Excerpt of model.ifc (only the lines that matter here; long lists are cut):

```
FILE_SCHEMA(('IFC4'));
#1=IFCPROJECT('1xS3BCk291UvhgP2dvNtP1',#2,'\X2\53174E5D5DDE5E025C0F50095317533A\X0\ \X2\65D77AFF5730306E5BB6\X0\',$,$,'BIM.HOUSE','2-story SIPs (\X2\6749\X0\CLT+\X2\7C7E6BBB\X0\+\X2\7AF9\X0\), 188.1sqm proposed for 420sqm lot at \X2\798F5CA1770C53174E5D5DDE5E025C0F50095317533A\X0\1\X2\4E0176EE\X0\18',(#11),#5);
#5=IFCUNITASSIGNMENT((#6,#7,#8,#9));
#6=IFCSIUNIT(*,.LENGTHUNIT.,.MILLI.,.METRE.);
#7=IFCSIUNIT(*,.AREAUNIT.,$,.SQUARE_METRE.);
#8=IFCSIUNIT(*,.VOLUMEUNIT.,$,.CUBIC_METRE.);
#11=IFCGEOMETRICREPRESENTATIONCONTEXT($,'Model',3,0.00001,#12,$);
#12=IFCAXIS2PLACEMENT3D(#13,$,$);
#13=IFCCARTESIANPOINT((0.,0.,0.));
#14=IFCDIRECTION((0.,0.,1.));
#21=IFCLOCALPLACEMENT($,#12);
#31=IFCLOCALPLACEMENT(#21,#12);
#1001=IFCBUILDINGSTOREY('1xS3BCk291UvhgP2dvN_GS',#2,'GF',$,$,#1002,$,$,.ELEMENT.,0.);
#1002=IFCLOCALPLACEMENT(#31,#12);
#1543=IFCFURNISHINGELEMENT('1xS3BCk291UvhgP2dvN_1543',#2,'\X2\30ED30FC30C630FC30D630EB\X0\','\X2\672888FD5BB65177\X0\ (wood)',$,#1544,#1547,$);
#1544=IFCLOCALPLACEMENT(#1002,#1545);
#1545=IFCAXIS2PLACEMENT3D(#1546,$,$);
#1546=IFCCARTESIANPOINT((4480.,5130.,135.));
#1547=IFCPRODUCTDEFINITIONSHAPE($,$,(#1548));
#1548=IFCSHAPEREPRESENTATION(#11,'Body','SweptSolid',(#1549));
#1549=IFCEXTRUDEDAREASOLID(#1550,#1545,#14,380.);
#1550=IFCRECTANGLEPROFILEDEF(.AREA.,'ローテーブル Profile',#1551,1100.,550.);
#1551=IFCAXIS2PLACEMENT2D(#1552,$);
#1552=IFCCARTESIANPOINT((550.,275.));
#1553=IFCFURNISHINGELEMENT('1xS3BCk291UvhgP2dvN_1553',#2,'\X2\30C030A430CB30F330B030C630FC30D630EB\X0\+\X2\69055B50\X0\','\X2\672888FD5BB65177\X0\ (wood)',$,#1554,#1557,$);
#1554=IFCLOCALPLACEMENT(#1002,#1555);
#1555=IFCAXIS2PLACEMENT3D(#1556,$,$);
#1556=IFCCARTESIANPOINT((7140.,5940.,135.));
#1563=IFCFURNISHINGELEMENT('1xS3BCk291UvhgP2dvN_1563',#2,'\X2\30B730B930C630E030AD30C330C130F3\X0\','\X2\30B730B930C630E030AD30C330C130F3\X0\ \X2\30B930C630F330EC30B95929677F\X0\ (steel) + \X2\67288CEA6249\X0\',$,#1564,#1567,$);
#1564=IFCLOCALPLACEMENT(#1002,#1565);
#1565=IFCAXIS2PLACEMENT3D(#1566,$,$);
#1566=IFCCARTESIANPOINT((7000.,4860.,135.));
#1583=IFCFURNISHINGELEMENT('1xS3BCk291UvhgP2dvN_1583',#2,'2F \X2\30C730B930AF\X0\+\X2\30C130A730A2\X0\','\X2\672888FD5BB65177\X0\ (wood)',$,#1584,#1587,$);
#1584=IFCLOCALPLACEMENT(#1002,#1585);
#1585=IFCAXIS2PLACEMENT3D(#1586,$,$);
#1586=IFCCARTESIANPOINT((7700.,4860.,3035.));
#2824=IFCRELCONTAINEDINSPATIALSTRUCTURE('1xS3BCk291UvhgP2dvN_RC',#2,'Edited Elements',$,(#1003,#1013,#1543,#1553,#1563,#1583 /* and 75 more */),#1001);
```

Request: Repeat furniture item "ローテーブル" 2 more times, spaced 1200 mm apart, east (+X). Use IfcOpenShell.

```python
import numpy as np
import ifcopenshell
import ifcopenshell.api.geometry
import ifcopenshell.api.root
import ifcopenshell.util.element
import ifcopenshell.util.placement
import ifcopenshell.util.unit

model = ifcopenshell.open("model.ifc")
unit_scale = ifcopenshell.util.unit.calculate_unit_scale(model)


def reuse_history(source, copy):
    """copy_class also copies each property set's owner history, people and application; keep the originals."""
    for rel in copy.IsDefinedBy:
        if rel.is_a("IfcRelDefinesByProperties") and (history := rel.RelatingPropertyDefinition.OwnerHistory):
            rel.RelatingPropertyDefinition.OwnerHistory = source.OwnerHistory
            ifcopenshell.util.element.remove_deep2(model, history)


source = model.by_guid("1xS3BCk291UvhgP2dvN_1543")
base = ifcopenshell.util.placement.get_local_placement(source.ObjectPlacement)
step = np.array([1.0, 0.0, 0.0]) * 1.2 / unit_scale

for i in range(1, 3):
    copy = ifcopenshell.api.root.copy_class(model, product=source)
    copy.Representation = ifcopenshell.util.element.copy_deep(
        model, source.Representation, exclude=["IfcGeometricRepresentationContext", "IfcRepresentationMap"]
    )
    reuse_history(source, copy)
    matrix = base.copy()
    matrix[:3, 3] += i * step
    print("added at", matrix[:3, 3].round(3) + 0.0)
    ifcopenshell.api.geometry.edit_object_placement(model, product=copy, matrix=matrix, is_si=False)

model.write("model-out.ifc")
```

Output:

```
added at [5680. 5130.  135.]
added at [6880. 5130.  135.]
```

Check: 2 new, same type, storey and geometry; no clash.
